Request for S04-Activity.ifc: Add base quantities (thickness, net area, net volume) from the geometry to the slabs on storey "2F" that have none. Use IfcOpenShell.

First a look at what the model holds.

```python
import ifcopenshell
import ifcopenshell.util.element
import ifcopenshell.util.unit

model = ifcopenshell.open("S04-Activity.ifc")
print(model.schema)
for unit_type in ("LENGTHUNIT", "AREAUNIT", "VOLUMEUNIT"):
    print(unit_type, ifcopenshell.util.unit.calculate_unit_scale(model, unit_type))
storey = next(s for s in model.by_type("IfcBuildingStorey") if s.Name == "2F")
slabs = [e for e in ifcopenshell.util.element.get_decomposition(storey) if e.is_a("IfcSlab")]
for e in sorted(slabs, key=lambda e: e.id()):
    print(e.id(), e.is_a(), e.Name, list(ifcopenshell.util.element.get_psets(e, qtos_only=True)), sep=" | ")
```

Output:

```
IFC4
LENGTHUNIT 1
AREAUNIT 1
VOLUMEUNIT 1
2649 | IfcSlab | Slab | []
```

```python
import ifcopenshell
import ifcopenshell.api.pset
import ifcopenshell.geom
import ifcopenshell.util.element
import ifcopenshell.util.shape
import ifcopenshell.util.unit

model = ifcopenshell.open("S04-Activity.ifc")
unit_scale = ifcopenshell.util.unit.calculate_unit_scale(model)
area_scale = ifcopenshell.util.unit.calculate_unit_scale(model, "AREAUNIT")
volume_scale = ifcopenshell.util.unit.calculate_unit_scale(model, "VOLUMEUNIT")
settings = ifcopenshell.geom.settings()

storey = next(s for s in model.by_type("IfcBuildingStorey") if s.Name == "2F")
slabs = [e for e in ifcopenshell.util.element.get_decomposition(storey) if e.is_a("IfcSlab")]

for e in sorted(slabs, key=lambda e: e.id()):
    if ifcopenshell.util.element.get_psets(e, qtos_only=True, should_inherit=False):
        continue
    # Geometry comes back in metres, in the element's own axes.
    shape = ifcopenshell.geom.create_shape(settings, e)
    values = {
        "Width": ifcopenshell.util.shape.get_z(shape.geometry) / unit_scale,
        "NetArea": ifcopenshell.util.shape.get_footprint_area(shape.geometry) / area_scale,
        "NetVolume": ifcopenshell.util.shape.get_volume(shape.geometry) / volume_scale,
    }
    qto = ifcopenshell.api.pset.add_qto(model, product=e, name="Qto_SlabBaseQuantities")
    ifcopenshell.api.pset.edit_qto(model, qto=qto, properties=values)
    print(e.id(), {k: round(v, 3) for k, v in values.items()})

model.write("S04-Activity_rev.ifc")
```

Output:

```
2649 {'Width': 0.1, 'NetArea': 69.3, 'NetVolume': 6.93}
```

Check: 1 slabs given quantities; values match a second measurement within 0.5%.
